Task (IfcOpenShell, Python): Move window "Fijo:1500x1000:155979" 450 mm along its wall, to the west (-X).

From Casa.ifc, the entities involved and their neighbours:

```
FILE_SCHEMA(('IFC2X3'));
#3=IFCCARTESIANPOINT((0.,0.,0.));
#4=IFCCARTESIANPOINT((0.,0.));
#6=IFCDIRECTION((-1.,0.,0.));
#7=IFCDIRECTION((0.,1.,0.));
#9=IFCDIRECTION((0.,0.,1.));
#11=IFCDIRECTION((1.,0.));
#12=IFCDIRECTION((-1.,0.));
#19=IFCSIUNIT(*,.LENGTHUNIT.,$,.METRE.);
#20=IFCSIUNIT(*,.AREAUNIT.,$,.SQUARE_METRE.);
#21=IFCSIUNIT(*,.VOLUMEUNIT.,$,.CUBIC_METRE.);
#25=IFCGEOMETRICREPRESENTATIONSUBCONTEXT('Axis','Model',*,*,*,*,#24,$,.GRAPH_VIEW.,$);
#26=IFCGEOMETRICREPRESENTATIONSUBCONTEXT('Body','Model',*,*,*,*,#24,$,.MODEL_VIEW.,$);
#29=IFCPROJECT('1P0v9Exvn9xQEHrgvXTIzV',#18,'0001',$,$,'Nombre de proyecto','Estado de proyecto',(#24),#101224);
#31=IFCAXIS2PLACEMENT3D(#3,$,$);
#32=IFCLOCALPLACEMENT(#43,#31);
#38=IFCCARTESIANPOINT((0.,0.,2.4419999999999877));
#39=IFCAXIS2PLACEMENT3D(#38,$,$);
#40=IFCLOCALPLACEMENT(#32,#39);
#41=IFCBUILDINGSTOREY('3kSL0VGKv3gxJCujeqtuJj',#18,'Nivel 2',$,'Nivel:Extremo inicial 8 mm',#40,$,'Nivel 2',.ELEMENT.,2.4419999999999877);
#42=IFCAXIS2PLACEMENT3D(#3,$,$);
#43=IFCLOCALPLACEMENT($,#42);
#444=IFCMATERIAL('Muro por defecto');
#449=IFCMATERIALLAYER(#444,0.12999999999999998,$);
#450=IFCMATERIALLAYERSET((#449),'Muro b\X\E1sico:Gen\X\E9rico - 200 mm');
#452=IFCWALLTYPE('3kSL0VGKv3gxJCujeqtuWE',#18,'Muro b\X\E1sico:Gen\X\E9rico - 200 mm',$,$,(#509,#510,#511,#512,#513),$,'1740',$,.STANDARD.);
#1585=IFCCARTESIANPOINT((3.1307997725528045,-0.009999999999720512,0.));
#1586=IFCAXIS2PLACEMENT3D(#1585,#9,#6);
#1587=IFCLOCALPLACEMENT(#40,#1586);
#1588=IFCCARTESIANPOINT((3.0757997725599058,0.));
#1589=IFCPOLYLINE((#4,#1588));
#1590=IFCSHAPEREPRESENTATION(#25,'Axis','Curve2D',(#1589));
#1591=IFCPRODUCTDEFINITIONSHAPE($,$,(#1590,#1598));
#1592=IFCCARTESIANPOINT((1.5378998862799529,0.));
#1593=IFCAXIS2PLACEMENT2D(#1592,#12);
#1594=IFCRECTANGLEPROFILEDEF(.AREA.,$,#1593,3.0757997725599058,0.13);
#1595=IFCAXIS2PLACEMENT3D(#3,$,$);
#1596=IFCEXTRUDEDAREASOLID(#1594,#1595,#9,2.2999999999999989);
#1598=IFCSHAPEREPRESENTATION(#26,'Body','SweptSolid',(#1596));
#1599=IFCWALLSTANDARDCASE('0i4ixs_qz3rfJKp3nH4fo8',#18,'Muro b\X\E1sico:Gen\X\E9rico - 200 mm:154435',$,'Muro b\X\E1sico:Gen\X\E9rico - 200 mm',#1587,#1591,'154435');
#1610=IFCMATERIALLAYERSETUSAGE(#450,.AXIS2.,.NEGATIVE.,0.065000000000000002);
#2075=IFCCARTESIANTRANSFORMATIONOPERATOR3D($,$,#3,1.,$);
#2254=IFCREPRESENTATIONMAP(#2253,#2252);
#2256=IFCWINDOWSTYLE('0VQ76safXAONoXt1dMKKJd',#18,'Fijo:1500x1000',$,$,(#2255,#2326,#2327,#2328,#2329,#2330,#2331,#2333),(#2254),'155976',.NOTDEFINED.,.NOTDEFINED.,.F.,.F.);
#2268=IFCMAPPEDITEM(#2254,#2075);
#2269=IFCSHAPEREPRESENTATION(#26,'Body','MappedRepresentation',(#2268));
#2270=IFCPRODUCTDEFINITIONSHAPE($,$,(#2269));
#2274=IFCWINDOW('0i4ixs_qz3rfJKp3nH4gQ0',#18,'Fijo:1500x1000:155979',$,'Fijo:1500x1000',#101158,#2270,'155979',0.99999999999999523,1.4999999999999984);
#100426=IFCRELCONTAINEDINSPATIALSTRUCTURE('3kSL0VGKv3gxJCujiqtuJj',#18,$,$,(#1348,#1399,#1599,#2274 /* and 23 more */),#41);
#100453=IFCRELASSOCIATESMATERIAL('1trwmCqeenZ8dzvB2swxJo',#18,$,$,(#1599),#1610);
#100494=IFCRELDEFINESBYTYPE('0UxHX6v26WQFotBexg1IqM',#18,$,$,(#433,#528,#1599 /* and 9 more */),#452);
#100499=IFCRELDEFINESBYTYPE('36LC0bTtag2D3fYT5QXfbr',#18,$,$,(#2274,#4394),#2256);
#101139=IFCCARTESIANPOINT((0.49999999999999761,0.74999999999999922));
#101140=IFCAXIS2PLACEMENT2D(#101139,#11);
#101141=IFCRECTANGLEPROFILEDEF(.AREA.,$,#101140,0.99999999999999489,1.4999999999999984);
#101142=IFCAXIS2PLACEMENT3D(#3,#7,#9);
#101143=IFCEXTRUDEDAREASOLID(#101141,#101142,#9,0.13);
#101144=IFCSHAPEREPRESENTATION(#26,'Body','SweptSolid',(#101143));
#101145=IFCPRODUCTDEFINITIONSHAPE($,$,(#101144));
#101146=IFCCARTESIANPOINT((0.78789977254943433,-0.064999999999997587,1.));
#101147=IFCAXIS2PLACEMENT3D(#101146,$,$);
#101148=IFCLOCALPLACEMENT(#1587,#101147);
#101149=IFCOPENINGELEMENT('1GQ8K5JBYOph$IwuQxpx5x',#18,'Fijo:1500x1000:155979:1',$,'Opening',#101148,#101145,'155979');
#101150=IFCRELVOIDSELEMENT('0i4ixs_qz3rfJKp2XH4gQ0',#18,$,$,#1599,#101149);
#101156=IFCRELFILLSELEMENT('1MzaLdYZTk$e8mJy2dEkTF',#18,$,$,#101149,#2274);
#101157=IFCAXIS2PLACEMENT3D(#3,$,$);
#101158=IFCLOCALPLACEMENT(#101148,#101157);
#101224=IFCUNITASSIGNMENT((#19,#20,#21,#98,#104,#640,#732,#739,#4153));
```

```python
import ifcopenshell
import ifcopenshell.api.geometry
import ifcopenshell.util.placement
import ifcopenshell.util.unit

model = ifcopenshell.open("Casa.ifc")
unit_scale = ifcopenshell.util.unit.calculate_unit_scale(model)

window = model.by_guid("0i4ixs_qz3rfJKp3nH4gQ0")
opening = window.FillsVoids[0].RelatingOpeningElement
wall = opening.VoidsElements[0].RelatingBuildingElement

wall_matrix = ifcopenshell.util.placement.get_local_placement(wall.ObjectPlacement)
shift = wall_matrix[:3, 0] * 0.45 / unit_scale
before = ifcopenshell.util.placement.get_local_placement(window.ObjectPlacement)[:3, 3].copy()

# The window is placed relative to its opening, so it follows when the opening moves.
matrix = ifcopenshell.util.placement.get_local_placement(opening.ObjectPlacement)
matrix[:3, 3] += shift
ifcopenshell.api.geometry.edit_object_placement(
    model, product=opening, matrix=matrix, is_si=False, should_transform_children=True
)

after = ifcopenshell.util.placement.get_local_placement(window.ObjectPlacement)[:3, 3]
print("window moved by", (after - before).round(3) + 0.0)

model.write("Casa_edited.ifc")
```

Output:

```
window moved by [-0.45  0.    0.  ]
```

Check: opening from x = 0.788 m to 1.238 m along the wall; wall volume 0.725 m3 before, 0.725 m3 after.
